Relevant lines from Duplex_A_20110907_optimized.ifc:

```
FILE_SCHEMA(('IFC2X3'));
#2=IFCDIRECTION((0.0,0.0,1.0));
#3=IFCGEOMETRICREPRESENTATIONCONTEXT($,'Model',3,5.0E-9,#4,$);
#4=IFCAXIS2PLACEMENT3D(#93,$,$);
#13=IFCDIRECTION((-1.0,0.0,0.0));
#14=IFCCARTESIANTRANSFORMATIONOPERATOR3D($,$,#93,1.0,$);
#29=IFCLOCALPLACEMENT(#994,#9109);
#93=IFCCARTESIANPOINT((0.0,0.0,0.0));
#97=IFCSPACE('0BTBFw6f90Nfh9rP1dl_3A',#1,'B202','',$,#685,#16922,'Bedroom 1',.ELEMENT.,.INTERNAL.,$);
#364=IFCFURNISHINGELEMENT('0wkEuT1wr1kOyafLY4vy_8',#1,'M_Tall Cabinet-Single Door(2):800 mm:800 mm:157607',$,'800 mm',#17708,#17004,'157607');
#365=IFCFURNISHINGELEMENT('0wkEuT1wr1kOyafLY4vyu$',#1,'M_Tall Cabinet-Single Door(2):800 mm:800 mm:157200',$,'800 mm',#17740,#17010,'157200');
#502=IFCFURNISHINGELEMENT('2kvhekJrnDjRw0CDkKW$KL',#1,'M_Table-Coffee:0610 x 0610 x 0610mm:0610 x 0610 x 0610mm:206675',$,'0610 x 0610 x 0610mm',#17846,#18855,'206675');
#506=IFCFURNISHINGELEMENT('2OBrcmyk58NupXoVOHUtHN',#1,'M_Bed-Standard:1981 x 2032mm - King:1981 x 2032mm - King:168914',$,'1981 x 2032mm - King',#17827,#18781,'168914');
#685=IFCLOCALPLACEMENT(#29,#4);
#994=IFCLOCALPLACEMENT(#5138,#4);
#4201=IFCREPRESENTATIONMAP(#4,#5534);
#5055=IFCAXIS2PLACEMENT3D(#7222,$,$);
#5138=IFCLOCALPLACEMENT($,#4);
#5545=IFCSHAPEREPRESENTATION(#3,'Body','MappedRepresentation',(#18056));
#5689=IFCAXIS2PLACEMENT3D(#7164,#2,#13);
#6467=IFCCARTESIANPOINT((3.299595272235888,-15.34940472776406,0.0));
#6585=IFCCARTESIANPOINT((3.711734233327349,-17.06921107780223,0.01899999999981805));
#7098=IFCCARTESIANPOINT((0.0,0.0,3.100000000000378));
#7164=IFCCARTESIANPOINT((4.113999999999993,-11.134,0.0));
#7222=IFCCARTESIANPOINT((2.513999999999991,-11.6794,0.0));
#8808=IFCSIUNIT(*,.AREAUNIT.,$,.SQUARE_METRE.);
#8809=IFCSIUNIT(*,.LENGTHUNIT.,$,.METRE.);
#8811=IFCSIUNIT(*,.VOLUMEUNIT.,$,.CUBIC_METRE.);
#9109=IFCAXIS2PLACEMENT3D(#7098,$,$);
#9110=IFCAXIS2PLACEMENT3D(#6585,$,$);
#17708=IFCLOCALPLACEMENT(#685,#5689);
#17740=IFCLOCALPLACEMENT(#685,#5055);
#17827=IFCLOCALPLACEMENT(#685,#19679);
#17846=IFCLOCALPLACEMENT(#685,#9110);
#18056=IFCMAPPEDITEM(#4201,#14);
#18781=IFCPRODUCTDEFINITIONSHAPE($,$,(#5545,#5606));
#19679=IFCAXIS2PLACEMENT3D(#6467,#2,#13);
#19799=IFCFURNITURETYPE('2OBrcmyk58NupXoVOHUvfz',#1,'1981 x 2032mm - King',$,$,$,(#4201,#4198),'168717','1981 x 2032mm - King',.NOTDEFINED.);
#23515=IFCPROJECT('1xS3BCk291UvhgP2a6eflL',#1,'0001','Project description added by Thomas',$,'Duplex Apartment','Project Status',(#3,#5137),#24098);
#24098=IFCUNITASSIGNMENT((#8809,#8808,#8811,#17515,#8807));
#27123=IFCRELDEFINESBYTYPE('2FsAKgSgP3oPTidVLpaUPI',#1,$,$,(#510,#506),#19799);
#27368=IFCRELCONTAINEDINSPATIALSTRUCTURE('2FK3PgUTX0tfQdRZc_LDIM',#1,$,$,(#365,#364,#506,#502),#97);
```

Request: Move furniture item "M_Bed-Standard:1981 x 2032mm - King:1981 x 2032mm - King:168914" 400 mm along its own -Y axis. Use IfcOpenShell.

```python
import ifcopenshell
import ifcopenshell.api.geometry
import ifcopenshell.util.placement
import ifcopenshell.util.unit

model = ifcopenshell.open("Duplex_A_20110907_optimized.ifc")
unit_scale = ifcopenshell.util.unit.calculate_unit_scale(model)

item = model.by_guid("2OBrcmyk58NupXoVOHUtHN")
matrix = ifcopenshell.util.placement.get_local_placement(item.ObjectPlacement)
matrix[:3, 3] -= matrix[:3, 1] * 0.4 / unit_scale
ifcopenshell.api.geometry.edit_object_placement(model, product=item, matrix=matrix, is_si=False)

print(ifcopenshell.util.placement.get_local_placement(item.ObjectPlacement).round(3) + 0.0)

model.write("Duplex_A_20110907_optimized_rev.ifc")
```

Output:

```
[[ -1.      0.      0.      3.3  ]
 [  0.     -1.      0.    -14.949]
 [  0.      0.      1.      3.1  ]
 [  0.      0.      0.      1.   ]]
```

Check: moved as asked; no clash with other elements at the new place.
